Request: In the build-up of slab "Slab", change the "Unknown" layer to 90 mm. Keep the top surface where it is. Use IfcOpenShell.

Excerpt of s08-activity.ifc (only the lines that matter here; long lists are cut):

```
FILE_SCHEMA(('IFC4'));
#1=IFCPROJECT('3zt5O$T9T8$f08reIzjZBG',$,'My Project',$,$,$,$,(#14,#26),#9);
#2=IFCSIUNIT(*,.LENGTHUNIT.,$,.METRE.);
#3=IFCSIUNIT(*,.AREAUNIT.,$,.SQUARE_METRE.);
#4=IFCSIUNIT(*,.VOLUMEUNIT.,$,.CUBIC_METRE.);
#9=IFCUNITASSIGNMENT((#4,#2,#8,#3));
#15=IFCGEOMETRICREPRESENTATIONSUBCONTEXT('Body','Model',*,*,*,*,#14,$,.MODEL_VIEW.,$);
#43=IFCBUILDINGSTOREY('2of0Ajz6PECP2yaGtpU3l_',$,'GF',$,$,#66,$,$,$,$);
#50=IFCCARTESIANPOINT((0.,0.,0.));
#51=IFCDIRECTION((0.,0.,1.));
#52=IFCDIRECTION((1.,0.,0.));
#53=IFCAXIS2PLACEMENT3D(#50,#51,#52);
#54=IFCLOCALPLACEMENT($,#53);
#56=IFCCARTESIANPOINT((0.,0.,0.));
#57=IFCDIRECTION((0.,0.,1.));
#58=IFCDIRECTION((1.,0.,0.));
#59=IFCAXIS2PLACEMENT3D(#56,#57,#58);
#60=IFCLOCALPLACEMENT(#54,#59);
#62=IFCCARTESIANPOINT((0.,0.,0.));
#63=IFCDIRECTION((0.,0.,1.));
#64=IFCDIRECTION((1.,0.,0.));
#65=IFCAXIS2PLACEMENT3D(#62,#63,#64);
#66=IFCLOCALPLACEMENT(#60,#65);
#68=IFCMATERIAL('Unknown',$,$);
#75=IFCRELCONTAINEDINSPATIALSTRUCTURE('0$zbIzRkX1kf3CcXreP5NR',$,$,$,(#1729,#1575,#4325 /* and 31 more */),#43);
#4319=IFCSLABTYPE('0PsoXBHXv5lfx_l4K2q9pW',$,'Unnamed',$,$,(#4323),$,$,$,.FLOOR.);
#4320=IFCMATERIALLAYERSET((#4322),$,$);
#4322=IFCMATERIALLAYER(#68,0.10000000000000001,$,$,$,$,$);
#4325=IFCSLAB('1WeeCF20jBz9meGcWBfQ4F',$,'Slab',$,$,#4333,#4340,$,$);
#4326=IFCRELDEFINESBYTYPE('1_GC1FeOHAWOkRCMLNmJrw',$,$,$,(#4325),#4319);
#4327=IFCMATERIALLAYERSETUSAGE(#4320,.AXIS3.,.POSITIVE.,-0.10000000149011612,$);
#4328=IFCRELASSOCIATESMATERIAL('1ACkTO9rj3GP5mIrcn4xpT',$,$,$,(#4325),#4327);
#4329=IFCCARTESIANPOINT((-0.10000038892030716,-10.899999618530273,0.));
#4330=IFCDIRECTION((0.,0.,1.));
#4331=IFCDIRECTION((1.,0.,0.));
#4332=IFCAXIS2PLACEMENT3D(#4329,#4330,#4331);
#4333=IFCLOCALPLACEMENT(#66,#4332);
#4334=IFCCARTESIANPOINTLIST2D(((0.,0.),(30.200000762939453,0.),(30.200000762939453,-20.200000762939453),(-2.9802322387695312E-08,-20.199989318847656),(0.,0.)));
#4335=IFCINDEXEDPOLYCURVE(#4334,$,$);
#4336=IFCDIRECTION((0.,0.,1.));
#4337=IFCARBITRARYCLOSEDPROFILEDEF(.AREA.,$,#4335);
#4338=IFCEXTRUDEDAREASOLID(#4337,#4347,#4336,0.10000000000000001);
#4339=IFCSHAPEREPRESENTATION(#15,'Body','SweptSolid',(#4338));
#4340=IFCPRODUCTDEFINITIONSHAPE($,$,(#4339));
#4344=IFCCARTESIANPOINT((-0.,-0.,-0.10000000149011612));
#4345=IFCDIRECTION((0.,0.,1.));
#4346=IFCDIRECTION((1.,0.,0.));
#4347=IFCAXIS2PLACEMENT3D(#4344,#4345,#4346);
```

```python
import ifcopenshell
import ifcopenshell.util.element
import ifcopenshell.util.representation

model = ifcopenshell.open("s08-activity.ifc")

layer_set = model.by_id(4320)
layer = next(l for l in layer_set.MaterialLayers if l.Material and l.Material.Name == "Unknown")
change = 0.09 - layer.LayerThickness
layer.LayerThickness += change

# Geometry does not follow the layer set by itself.
slabs = [e for e in ifcopenshell.util.element.get_elements_by_material(model, layer_set) if e.is_a("IfcSlab")]
for slab in sorted(slabs, key=lambda e: e.id()):
    body = ifcopenshell.util.representation.get_representation(slab, "Model", "Body")
    solid = body.Items[0]
    old_depth = solid.Depth
    solid.Depth += change
    # Extruded upwards: lower the start of the extrusion so the top stays.
    x, y, z = solid.Position.Location.Coordinates
    solid.Position.Location = model.createIfcCartesianPoint((x, y, z - change))
    print(slab.id(), f"{old_depth:g} -> {solid.Depth:g}")

# The layers are counted up from the underside, which has moved.
for usage in {ifcopenshell.util.element.get_material(slab) for slab in slabs}:
    usage.OffsetFromReferenceLine -= change

model.write("s08-activity_updated.ifc")
```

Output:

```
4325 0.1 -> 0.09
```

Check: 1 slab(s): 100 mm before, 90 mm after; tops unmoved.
